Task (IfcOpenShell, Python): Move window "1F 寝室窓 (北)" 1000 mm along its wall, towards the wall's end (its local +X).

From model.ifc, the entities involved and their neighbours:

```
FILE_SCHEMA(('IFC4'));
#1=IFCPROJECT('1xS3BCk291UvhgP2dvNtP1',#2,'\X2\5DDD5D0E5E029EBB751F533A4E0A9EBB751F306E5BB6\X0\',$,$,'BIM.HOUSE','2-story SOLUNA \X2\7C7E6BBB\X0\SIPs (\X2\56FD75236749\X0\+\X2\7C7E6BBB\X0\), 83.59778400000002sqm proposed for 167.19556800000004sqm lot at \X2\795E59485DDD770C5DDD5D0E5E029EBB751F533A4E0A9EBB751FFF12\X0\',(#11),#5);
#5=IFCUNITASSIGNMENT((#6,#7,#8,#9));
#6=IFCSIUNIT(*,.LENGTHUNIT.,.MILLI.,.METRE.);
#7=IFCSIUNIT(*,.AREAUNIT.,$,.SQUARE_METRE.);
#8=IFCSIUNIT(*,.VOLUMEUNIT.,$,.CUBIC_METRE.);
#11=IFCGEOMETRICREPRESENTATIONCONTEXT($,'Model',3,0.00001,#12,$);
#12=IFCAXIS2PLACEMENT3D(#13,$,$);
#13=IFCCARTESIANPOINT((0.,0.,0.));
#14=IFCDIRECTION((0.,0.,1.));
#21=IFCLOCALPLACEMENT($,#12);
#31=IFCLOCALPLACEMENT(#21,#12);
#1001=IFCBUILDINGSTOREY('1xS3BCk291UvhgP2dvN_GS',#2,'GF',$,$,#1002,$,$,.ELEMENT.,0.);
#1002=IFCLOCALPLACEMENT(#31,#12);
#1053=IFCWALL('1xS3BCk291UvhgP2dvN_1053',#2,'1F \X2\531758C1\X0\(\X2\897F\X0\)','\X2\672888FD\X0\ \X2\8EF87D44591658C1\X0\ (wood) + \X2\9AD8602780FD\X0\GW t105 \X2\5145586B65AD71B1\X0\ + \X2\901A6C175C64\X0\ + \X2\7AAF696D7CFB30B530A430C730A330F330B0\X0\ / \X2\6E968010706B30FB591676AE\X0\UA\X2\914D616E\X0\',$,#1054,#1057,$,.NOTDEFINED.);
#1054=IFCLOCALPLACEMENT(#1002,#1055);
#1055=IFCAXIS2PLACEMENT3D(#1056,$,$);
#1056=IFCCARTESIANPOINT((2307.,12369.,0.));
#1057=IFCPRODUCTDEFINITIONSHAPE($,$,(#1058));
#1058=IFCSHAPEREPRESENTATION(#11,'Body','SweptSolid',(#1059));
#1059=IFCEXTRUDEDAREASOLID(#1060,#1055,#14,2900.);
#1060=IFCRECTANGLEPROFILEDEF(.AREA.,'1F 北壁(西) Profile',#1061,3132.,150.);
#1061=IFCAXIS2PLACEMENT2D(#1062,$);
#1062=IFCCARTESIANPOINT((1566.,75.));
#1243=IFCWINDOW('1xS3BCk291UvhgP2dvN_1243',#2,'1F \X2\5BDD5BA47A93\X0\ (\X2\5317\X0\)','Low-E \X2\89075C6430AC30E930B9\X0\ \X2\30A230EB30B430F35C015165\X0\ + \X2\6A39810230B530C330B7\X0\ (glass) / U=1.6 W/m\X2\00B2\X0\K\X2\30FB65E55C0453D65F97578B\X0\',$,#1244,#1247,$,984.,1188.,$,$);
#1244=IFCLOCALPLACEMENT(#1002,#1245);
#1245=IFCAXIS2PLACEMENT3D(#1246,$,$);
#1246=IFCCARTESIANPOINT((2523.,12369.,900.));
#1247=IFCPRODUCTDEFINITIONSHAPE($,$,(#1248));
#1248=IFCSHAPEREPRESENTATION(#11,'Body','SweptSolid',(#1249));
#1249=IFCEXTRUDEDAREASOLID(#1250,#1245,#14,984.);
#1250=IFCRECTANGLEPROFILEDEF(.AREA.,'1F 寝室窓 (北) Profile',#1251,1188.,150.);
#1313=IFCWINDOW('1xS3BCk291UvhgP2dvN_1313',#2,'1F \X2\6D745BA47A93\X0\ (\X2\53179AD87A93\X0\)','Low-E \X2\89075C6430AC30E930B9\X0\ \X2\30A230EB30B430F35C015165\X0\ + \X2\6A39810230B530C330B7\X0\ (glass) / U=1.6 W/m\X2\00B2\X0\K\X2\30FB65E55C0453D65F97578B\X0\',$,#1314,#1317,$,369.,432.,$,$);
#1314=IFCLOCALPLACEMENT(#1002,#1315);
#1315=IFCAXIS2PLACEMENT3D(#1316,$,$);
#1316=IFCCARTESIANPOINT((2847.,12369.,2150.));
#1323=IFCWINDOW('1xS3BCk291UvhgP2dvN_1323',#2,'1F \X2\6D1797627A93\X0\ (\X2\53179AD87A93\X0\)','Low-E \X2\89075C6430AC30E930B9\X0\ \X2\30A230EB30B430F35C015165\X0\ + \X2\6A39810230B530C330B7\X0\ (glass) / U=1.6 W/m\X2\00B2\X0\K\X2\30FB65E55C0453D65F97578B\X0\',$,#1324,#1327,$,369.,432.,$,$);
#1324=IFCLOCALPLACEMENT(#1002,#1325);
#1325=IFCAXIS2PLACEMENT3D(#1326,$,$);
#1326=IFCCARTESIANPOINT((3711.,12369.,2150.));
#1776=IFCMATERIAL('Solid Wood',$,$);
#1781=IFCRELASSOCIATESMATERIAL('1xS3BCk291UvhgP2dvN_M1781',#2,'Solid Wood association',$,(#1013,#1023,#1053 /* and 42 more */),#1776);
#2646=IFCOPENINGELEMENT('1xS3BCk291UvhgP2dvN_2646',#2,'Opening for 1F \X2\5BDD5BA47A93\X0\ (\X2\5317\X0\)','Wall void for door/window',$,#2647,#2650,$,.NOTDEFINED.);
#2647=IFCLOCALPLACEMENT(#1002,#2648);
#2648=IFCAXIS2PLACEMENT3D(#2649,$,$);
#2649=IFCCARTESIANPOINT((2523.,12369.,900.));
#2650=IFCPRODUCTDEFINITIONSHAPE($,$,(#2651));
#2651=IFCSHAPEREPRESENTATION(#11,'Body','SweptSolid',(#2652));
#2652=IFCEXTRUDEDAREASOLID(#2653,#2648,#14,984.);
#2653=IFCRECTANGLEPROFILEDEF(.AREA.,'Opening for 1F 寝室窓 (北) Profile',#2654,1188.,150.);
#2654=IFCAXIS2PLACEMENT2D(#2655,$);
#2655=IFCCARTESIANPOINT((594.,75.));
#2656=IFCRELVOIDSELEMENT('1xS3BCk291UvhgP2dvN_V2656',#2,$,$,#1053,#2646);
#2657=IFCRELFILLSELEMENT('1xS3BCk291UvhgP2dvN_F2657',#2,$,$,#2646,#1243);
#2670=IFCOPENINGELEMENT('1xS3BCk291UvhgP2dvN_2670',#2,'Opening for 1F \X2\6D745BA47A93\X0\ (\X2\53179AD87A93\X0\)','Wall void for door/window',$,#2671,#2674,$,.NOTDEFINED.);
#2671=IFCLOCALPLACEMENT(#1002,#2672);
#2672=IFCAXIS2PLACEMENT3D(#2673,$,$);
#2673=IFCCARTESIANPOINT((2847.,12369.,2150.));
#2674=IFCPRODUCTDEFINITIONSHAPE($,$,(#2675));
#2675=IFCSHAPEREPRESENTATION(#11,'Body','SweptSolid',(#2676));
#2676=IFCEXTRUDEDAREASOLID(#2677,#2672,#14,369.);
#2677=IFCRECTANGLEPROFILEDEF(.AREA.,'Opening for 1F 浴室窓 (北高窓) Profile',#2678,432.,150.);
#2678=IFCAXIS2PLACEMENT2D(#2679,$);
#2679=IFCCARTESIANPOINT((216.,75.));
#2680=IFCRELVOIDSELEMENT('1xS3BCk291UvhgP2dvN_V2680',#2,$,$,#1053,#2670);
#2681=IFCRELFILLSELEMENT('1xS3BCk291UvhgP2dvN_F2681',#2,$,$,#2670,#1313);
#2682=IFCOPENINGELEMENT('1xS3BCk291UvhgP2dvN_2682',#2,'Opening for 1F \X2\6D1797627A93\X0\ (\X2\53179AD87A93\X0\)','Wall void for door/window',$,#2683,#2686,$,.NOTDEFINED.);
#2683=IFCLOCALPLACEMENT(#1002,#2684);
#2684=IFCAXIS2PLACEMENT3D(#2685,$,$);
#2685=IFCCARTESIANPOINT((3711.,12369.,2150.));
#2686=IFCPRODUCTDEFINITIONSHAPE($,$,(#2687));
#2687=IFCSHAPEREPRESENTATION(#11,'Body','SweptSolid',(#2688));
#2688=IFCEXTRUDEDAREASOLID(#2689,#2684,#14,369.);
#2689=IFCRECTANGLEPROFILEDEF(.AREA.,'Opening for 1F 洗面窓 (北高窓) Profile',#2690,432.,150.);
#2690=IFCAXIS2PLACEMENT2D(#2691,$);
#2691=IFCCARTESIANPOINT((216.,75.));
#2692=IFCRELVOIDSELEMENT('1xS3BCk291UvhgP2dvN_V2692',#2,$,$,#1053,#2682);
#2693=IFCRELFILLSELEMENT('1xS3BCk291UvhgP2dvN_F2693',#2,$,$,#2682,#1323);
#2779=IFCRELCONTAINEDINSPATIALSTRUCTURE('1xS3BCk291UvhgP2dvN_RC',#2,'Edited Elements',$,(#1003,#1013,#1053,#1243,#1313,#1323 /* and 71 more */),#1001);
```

```python
import ifcopenshell
import ifcopenshell.api.geometry
import ifcopenshell.util.placement

model = ifcopenshell.open("model.ifc")

window = model.by_id(1243)
opening = window.FillsVoids[0].RelatingOpeningElement
wall = opening.VoidsElements[0].RelatingBuildingElement

wall_matrix = ifcopenshell.util.placement.get_local_placement(wall.ObjectPlacement)
shift = wall_matrix[:3, 0] * 1000.0
before = ifcopenshell.util.placement.get_local_placement(window.ObjectPlacement)[:3, 3].copy()

# The window is not placed relative to its opening, so move both.
for product in (opening, window):
    matrix = ifcopenshell.util.placement.get_local_placement(product.ObjectPlacement)
    matrix[:3, 3] += shift
    ifcopenshell.api.geometry.edit_object_placement(model, product=product, matrix=matrix, is_si=False)

after = ifcopenshell.util.placement.get_local_placement(window.ObjectPlacement)[:3, 3]
print("window moved by", (after - before).round(3) + 0.0)

model.write("model_rev.ifc")
```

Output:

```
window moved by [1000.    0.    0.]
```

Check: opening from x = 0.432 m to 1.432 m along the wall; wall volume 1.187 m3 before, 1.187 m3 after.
